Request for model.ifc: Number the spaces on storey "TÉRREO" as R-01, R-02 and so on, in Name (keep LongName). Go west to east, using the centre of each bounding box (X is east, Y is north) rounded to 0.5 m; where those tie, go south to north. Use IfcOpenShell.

First a look at what the model holds.

```python
import ifcopenshell
import ifcopenshell.util.element
import ifcopenshell.util.placement

model = ifcopenshell.open("model.ifc")
print(model.schema)
storey = next(s for s in model.by_type("IfcBuildingStorey") if s.Name == "TÉRREO")
spaces = [e for e in ifcopenshell.util.element.get_decomposition(storey) if e.is_a("IfcSpace")]
for e in sorted(spaces, key=lambda e: e.id()):
    origin = ifcopenshell.util.placement.get_local_placement(e.ObjectPlacement)[:3, 3]
    print(e.id(), e.Name, e.LongName, origin.round(2) + 0.0, sep=" | ")
```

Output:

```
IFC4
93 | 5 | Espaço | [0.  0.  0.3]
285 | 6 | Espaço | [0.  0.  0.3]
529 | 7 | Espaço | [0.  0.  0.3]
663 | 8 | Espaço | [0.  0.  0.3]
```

```python
import ifcopenshell
import ifcopenshell.geom
import ifcopenshell.util.element
import ifcopenshell.util.shape

model = ifcopenshell.open("model.ifc")
settings = ifcopenshell.geom.settings()
settings.set("use-world-coords", True)


def centre(element):
    shape = ifcopenshell.geom.create_shape(settings, element)
    return ifcopenshell.util.shape.get_bbox_centroid(shape.geometry)


storey = next(s for s in model.by_type("IfcBuildingStorey") if s.Name == "TÉRREO")
spaces = [e for e in ifcopenshell.util.element.get_decomposition(storey) if e.is_a("IfcSpace")]

# Insertion points can sit at a corner or the storey origin, so sort by the geometry (in metres).
centres = {e: centre(e) for e in spaces}
spaces.sort(key=lambda e: (round(centres[e][0] / 0.5), centres[e][1]))

for i, e in enumerate(spaces, start=1):
    number = f"R-{i:02d}"
    e.Name = number
    print(e.id(), number)

model.write("model_updated.ifc")
```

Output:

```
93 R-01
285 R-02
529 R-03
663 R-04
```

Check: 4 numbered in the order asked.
